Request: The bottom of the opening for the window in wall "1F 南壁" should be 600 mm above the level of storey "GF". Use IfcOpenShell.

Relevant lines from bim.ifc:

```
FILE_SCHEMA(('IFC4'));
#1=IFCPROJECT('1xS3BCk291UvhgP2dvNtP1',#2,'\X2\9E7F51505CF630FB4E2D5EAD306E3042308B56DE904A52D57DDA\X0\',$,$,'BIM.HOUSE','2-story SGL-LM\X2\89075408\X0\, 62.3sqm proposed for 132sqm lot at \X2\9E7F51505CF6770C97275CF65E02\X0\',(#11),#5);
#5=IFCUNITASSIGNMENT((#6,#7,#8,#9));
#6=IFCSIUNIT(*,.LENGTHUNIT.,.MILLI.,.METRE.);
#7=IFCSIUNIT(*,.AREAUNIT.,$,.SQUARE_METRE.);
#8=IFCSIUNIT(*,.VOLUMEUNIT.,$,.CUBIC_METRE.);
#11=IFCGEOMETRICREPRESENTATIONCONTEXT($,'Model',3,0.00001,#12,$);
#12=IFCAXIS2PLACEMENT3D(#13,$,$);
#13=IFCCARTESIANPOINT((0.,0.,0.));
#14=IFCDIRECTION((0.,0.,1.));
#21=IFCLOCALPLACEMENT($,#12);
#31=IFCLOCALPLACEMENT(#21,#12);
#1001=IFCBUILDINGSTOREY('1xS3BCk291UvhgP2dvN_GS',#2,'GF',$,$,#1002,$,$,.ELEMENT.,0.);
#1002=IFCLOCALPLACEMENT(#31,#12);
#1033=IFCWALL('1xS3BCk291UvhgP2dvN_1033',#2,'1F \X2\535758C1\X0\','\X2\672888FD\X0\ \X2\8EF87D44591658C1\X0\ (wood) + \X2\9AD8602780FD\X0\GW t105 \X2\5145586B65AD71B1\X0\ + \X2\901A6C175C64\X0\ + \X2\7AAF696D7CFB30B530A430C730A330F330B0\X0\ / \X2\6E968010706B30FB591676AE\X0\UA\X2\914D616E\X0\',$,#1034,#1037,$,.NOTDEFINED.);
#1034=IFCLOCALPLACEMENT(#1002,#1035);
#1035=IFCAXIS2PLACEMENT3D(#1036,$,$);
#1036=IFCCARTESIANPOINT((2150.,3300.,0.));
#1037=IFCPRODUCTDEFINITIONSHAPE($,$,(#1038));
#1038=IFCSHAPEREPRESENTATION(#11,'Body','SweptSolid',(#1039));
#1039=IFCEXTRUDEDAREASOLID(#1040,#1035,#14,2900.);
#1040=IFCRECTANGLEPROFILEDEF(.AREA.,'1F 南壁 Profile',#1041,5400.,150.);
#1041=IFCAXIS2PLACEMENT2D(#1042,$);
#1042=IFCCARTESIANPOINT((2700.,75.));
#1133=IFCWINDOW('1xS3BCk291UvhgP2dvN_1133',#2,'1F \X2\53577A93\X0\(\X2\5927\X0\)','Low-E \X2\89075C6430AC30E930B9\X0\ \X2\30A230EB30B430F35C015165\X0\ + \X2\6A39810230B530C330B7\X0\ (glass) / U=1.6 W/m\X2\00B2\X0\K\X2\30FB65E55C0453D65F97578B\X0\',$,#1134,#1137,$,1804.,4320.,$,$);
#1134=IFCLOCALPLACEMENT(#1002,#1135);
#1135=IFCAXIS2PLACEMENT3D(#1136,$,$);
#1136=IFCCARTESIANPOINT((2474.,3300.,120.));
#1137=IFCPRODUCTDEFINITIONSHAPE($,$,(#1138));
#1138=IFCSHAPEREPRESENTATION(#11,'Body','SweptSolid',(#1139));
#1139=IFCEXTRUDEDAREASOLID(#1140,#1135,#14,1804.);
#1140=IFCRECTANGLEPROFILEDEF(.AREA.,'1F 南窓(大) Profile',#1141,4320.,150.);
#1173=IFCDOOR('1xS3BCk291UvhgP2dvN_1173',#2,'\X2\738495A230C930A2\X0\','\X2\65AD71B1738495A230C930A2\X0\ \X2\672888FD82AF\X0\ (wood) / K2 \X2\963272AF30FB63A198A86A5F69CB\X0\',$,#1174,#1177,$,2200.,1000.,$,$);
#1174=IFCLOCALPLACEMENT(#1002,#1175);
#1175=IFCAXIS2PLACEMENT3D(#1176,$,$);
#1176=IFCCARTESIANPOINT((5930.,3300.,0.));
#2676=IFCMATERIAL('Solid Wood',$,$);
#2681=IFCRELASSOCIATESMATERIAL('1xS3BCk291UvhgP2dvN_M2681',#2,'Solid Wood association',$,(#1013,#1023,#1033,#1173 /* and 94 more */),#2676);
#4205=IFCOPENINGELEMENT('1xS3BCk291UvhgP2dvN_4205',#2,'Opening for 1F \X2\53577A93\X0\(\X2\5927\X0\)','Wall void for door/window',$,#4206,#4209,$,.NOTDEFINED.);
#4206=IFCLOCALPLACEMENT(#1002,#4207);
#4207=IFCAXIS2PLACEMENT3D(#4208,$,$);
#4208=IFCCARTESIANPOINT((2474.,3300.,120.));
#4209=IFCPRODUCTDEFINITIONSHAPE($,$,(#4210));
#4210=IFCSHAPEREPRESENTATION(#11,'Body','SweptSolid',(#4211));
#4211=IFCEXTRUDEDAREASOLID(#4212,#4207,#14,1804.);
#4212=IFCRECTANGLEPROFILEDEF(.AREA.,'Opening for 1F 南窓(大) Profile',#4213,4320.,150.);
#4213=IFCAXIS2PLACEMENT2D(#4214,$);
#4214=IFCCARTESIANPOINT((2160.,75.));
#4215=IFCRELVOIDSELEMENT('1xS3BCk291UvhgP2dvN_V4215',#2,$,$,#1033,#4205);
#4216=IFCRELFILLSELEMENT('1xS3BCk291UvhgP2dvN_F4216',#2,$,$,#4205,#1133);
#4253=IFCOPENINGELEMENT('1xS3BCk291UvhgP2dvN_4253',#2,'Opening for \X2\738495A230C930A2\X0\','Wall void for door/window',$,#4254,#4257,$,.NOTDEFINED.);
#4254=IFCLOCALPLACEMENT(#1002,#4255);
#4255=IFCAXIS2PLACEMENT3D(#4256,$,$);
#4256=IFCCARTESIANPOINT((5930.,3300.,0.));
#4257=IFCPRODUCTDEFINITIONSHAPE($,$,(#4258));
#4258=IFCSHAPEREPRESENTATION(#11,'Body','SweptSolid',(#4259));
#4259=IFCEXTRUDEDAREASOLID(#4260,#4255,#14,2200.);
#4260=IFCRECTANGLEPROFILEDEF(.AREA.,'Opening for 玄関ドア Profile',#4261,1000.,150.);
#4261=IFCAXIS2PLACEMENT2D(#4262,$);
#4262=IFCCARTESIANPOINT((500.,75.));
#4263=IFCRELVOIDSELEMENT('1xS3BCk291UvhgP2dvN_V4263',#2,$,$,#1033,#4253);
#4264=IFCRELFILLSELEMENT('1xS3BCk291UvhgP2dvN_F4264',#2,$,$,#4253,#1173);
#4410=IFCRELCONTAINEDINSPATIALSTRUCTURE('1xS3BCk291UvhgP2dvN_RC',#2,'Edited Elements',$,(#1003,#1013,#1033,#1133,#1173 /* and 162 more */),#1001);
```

```python
import numpy as np
import ifcopenshell
import ifcopenshell.api.geometry
import ifcopenshell.geom
import ifcopenshell.util.element
import ifcopenshell.util.placement
import ifcopenshell.util.shape
import ifcopenshell.util.unit

model = ifcopenshell.open("bim.ifc")
unit_scale = ifcopenshell.util.unit.calculate_unit_scale(model)

window = model.by_id(1133)
opening = window.FillsVoids[0].RelatingOpeningElement
storey = ifcopenshell.util.element.get_container(window, ifc_class="IfcBuildingStorey")
level = ifcopenshell.util.placement.get_local_placement(storey.ObjectPlacement)[2, 3]

# The opening's origin need not be at the sill, so measure its lowest point.
shape = ifcopenshell.geom.create_shape(ifcopenshell.geom.settings(), opening)
bottom = ifcopenshell.util.shape.get_shape_bottom_elevation(shape, shape.geometry) / unit_scale
dz = level + 600.0 - bottom

shift = np.array([0.0, 0.0, dz])
# The window is not placed relative to its opening, so move both.
for product in (opening, window):
    matrix = ifcopenshell.util.placement.get_local_placement(product.ObjectPlacement)
    matrix[:3, 3] += shift
    ifcopenshell.api.geometry.edit_object_placement(model, product=product, matrix=matrix, is_si=False)

print(f"moved by {dz * unit_scale:+.3f} m")

model.write("bim-out.ifc")
```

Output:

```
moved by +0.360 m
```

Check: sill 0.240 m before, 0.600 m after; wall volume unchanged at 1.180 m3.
